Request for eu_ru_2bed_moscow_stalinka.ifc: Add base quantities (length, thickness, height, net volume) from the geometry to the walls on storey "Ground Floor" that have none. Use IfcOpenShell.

First a look at what the model holds.

```python
import ifcopenshell
import ifcopenshell.util.element
import ifcopenshell.util.unit

model = ifcopenshell.open("eu_ru_2bed_moscow_stalinka.ifc")
print(model.schema)
for unit_type in ("LENGTHUNIT", "AREAUNIT", "VOLUMEUNIT"):
    print(unit_type, ifcopenshell.util.unit.calculate_unit_scale(model, unit_type))
storey = next(s for s in model.by_type("IfcBuildingStorey") if s.Name == "Ground Floor")
walls = [e for e in ifcopenshell.util.element.get_decomposition(storey) if e.is_a("IfcWall")]
for e in sorted(walls, key=lambda e: e.id()):
    print(e.id(), e.is_a(), e.Name, list(ifcopenshell.util.element.get_psets(e, qtos_only=True)), sep=" | ")
```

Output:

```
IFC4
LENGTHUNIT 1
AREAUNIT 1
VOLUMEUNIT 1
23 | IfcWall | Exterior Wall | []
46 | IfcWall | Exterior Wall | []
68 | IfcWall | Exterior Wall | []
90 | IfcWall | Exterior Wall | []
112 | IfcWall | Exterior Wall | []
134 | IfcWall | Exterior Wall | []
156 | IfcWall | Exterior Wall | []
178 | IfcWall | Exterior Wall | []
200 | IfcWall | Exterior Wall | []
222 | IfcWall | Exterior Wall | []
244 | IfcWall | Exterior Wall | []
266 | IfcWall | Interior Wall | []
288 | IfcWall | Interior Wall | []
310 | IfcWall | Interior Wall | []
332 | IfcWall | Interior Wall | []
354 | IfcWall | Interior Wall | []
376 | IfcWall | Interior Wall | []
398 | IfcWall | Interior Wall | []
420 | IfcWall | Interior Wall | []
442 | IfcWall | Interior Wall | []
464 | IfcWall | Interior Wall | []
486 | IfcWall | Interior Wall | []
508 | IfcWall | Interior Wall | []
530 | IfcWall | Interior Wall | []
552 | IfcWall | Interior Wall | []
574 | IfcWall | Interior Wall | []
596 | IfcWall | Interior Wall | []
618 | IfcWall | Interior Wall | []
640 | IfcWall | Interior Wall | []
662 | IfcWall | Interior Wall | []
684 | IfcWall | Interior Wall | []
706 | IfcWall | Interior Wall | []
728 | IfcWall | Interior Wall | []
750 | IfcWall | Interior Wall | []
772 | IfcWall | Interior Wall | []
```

```python
import ifcopenshell
import ifcopenshell.api.pset
import ifcopenshell.geom
import ifcopenshell.util.element
import ifcopenshell.util.shape
import ifcopenshell.util.unit

model = ifcopenshell.open("eu_ru_2bed_moscow_stalinka.ifc")
unit_scale = ifcopenshell.util.unit.calculate_unit_scale(model)
volume_scale = ifcopenshell.util.unit.calculate_unit_scale(model, "VOLUMEUNIT")
settings = ifcopenshell.geom.settings()

storey = next(s for s in model.by_type("IfcBuildingStorey") if s.Name == "Ground Floor")
walls = [e for e in ifcopenshell.util.element.get_decomposition(storey) if e.is_a("IfcWall")]

for e in sorted(walls, key=lambda e: e.id()):
    if ifcopenshell.util.element.get_psets(e, qtos_only=True, should_inherit=False):
        continue
    # Geometry comes back in metres, in the element's own axes.
    shape = ifcopenshell.geom.create_shape(settings, e)
    values = {
        "Length": ifcopenshell.util.shape.get_x(shape.geometry) / unit_scale,
        "Width": ifcopenshell.util.shape.get_y(shape.geometry) / unit_scale,
        "Height": ifcopenshell.util.shape.get_z(shape.geometry) / unit_scale,
        "NetVolume": ifcopenshell.util.shape.get_volume(shape.geometry) / volume_scale,
    }
    qto = ifcopenshell.api.pset.add_qto(model, product=e, name="Qto_WallBaseQuantities")
    ifcopenshell.api.pset.edit_qto(model, qto=qto, properties=values)
    print(e.id(), {k: round(v, 3) for k, v in values.items()})

model.write("eu_ru_2bed_moscow_stalinka_edited.ifc")
```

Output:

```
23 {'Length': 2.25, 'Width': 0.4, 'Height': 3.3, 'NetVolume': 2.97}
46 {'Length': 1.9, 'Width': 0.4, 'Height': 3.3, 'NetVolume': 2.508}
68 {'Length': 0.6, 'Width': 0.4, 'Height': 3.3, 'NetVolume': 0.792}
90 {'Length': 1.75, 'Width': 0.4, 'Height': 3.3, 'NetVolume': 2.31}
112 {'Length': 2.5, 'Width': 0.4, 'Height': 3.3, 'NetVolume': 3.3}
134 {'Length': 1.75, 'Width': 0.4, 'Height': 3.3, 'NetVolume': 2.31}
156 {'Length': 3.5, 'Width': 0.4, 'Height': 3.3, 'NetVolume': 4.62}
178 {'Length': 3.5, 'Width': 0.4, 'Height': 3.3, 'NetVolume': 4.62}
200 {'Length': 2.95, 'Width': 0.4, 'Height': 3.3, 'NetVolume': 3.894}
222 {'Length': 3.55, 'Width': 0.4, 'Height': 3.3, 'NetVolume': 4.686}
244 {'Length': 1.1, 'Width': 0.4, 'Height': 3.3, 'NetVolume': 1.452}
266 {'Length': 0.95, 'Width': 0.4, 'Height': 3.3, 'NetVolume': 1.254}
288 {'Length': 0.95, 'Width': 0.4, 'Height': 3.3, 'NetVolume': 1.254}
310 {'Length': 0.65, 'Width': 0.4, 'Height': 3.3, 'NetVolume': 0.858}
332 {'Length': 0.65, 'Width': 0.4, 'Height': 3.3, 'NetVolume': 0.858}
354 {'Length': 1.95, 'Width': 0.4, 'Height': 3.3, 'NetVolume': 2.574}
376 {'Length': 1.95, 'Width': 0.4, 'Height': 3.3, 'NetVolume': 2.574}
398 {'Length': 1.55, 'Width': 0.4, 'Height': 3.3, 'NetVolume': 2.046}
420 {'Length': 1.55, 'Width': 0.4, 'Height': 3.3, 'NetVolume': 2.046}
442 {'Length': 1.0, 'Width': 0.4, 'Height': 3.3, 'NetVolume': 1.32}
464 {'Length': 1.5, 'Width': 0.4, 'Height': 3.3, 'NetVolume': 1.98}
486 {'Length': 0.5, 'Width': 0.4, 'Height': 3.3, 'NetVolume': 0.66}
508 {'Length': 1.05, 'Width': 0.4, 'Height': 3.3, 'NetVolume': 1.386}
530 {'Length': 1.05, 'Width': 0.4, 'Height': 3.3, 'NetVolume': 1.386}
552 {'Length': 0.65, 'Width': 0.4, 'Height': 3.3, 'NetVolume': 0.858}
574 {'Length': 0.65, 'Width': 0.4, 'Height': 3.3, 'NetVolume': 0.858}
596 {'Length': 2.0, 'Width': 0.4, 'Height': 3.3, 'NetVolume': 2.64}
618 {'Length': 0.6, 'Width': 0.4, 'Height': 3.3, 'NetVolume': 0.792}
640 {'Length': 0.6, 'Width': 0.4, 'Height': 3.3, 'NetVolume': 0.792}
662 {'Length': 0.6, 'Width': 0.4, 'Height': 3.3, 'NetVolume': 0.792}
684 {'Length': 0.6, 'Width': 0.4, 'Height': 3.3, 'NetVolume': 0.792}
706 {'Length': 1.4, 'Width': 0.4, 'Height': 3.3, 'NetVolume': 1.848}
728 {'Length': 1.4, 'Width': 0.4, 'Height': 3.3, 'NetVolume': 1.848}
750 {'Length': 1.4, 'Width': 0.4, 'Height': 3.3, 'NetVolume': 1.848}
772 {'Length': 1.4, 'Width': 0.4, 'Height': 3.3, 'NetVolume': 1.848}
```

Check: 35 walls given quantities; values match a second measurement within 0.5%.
